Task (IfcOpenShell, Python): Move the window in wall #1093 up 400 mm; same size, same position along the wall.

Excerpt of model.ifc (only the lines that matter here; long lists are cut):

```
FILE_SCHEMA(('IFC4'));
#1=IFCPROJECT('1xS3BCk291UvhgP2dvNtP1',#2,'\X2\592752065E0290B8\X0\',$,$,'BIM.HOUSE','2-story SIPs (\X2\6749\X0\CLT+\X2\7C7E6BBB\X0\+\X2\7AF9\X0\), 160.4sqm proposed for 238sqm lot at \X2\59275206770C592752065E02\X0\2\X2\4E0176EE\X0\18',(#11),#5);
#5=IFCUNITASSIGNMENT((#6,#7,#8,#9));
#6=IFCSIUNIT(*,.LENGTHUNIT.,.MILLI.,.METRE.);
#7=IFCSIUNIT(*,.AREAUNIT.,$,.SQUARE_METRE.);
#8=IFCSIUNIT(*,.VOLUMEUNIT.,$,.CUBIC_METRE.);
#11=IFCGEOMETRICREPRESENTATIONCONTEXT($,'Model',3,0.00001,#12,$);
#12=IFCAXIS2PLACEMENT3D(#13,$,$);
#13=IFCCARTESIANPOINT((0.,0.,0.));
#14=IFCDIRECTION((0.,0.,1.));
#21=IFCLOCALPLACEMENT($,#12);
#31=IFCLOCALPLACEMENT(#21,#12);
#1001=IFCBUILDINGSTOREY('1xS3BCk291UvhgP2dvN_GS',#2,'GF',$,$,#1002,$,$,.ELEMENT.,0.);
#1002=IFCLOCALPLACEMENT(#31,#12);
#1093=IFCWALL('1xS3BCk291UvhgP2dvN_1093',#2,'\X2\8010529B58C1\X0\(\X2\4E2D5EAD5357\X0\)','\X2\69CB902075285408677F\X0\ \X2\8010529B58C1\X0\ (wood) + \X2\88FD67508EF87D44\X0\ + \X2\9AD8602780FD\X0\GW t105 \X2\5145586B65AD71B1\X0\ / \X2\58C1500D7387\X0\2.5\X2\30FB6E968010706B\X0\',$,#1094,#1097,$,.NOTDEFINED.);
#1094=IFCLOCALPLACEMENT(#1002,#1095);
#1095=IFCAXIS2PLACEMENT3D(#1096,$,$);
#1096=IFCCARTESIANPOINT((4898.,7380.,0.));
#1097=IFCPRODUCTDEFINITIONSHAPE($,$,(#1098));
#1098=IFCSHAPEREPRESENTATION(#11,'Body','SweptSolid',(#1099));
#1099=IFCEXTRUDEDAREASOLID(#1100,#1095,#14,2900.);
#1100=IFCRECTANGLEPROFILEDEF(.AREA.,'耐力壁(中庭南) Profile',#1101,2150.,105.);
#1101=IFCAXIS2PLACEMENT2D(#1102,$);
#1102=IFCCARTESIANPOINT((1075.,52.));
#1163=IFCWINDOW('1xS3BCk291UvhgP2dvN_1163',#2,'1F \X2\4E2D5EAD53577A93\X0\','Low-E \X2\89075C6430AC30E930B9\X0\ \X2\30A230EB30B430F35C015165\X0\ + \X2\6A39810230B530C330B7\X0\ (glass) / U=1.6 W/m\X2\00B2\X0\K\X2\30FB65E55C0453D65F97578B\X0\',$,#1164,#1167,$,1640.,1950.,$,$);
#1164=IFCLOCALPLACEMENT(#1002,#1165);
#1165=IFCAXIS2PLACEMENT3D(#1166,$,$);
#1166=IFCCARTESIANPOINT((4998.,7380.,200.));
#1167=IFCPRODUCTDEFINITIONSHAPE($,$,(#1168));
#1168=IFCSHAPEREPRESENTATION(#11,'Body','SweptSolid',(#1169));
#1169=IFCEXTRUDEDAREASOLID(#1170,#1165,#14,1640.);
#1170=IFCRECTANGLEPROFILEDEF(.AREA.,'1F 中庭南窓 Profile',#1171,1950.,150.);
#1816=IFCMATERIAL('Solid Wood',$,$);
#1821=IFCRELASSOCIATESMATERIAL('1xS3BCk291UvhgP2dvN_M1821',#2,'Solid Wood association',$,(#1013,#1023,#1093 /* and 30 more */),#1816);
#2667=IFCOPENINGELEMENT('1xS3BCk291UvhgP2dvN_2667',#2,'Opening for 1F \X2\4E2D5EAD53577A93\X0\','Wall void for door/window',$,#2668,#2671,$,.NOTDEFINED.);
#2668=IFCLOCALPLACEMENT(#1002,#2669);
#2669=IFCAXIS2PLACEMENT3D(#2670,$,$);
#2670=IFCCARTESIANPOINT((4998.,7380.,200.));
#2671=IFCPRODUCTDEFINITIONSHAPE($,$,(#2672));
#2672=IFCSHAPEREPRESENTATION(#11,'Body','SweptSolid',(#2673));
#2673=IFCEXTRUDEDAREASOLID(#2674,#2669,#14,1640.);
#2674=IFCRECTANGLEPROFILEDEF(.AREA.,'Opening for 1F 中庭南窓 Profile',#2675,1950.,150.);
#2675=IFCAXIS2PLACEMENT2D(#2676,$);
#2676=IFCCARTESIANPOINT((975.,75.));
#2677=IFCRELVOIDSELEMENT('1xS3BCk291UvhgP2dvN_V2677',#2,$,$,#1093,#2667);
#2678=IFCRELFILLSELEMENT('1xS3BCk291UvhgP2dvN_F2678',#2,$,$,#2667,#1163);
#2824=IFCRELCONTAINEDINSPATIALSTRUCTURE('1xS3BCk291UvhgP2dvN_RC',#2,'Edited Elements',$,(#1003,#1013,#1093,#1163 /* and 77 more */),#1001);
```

```python
import numpy as np
import ifcopenshell
import ifcopenshell.api.geometry
import ifcopenshell.util.placement
import ifcopenshell.util.unit

model = ifcopenshell.open("model.ifc")
unit_scale = ifcopenshell.util.unit.calculate_unit_scale(model)

window = model.by_guid("1xS3BCk291UvhgP2dvN_1163")
opening = window.FillsVoids[0].RelatingOpeningElement
dz = 0.4 / unit_scale

shift = np.array([0.0, 0.0, dz])
# The window is not placed relative to its opening, so move both.
for product in (opening, window):
    matrix = ifcopenshell.util.placement.get_local_placement(product.ObjectPlacement)
    matrix[:3, 3] += shift
    ifcopenshell.api.geometry.edit_object_placement(model, product=product, matrix=matrix, is_si=False)

print(f"moved by {dz * unit_scale:+.3f} m")

model.write("model-out.ifc")
```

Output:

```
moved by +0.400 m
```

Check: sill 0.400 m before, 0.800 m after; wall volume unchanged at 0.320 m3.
